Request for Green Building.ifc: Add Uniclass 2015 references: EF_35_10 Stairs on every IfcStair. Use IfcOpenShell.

First a look at what the model holds.

```python
import ifcopenshell

model = ifcopenshell.open("Green Building.ifc")
print(model.schema)
print("classifications:", [c.Name for c in model.by_type("IfcClassification")])
for ifc_class in ("IfcDoor", "IfcRoof", "IfcStair", "IfcWall", "IfcWindow"):
    print(ifc_class, len(model.by_type(ifc_class)))
```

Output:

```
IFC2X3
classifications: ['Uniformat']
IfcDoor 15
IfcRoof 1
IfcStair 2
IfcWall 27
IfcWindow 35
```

```python
import ifcopenshell
import ifcopenshell.api.classification

model = ifcopenshell.open("Green Building.ifc")

# IFC2X3 requires Source and Edition and has no link from the project to the system.
system = model.create_entity("IfcClassification", Source="NBS", Edition="2015", Name="Uniclass 2015")

codes = {
    "IfcStair": ("EF_35_10", "Stairs"),
}
for ifc_class, (code, name) in codes.items():
    products = model.by_type(ifc_class)
    ifcopenshell.api.classification.add_reference(
        model, products=products, classification=system, identification=code, name=name
    )
    print(code, len(products))

model.write("Green Building_rev.ifc")
```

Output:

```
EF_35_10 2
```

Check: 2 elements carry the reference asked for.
